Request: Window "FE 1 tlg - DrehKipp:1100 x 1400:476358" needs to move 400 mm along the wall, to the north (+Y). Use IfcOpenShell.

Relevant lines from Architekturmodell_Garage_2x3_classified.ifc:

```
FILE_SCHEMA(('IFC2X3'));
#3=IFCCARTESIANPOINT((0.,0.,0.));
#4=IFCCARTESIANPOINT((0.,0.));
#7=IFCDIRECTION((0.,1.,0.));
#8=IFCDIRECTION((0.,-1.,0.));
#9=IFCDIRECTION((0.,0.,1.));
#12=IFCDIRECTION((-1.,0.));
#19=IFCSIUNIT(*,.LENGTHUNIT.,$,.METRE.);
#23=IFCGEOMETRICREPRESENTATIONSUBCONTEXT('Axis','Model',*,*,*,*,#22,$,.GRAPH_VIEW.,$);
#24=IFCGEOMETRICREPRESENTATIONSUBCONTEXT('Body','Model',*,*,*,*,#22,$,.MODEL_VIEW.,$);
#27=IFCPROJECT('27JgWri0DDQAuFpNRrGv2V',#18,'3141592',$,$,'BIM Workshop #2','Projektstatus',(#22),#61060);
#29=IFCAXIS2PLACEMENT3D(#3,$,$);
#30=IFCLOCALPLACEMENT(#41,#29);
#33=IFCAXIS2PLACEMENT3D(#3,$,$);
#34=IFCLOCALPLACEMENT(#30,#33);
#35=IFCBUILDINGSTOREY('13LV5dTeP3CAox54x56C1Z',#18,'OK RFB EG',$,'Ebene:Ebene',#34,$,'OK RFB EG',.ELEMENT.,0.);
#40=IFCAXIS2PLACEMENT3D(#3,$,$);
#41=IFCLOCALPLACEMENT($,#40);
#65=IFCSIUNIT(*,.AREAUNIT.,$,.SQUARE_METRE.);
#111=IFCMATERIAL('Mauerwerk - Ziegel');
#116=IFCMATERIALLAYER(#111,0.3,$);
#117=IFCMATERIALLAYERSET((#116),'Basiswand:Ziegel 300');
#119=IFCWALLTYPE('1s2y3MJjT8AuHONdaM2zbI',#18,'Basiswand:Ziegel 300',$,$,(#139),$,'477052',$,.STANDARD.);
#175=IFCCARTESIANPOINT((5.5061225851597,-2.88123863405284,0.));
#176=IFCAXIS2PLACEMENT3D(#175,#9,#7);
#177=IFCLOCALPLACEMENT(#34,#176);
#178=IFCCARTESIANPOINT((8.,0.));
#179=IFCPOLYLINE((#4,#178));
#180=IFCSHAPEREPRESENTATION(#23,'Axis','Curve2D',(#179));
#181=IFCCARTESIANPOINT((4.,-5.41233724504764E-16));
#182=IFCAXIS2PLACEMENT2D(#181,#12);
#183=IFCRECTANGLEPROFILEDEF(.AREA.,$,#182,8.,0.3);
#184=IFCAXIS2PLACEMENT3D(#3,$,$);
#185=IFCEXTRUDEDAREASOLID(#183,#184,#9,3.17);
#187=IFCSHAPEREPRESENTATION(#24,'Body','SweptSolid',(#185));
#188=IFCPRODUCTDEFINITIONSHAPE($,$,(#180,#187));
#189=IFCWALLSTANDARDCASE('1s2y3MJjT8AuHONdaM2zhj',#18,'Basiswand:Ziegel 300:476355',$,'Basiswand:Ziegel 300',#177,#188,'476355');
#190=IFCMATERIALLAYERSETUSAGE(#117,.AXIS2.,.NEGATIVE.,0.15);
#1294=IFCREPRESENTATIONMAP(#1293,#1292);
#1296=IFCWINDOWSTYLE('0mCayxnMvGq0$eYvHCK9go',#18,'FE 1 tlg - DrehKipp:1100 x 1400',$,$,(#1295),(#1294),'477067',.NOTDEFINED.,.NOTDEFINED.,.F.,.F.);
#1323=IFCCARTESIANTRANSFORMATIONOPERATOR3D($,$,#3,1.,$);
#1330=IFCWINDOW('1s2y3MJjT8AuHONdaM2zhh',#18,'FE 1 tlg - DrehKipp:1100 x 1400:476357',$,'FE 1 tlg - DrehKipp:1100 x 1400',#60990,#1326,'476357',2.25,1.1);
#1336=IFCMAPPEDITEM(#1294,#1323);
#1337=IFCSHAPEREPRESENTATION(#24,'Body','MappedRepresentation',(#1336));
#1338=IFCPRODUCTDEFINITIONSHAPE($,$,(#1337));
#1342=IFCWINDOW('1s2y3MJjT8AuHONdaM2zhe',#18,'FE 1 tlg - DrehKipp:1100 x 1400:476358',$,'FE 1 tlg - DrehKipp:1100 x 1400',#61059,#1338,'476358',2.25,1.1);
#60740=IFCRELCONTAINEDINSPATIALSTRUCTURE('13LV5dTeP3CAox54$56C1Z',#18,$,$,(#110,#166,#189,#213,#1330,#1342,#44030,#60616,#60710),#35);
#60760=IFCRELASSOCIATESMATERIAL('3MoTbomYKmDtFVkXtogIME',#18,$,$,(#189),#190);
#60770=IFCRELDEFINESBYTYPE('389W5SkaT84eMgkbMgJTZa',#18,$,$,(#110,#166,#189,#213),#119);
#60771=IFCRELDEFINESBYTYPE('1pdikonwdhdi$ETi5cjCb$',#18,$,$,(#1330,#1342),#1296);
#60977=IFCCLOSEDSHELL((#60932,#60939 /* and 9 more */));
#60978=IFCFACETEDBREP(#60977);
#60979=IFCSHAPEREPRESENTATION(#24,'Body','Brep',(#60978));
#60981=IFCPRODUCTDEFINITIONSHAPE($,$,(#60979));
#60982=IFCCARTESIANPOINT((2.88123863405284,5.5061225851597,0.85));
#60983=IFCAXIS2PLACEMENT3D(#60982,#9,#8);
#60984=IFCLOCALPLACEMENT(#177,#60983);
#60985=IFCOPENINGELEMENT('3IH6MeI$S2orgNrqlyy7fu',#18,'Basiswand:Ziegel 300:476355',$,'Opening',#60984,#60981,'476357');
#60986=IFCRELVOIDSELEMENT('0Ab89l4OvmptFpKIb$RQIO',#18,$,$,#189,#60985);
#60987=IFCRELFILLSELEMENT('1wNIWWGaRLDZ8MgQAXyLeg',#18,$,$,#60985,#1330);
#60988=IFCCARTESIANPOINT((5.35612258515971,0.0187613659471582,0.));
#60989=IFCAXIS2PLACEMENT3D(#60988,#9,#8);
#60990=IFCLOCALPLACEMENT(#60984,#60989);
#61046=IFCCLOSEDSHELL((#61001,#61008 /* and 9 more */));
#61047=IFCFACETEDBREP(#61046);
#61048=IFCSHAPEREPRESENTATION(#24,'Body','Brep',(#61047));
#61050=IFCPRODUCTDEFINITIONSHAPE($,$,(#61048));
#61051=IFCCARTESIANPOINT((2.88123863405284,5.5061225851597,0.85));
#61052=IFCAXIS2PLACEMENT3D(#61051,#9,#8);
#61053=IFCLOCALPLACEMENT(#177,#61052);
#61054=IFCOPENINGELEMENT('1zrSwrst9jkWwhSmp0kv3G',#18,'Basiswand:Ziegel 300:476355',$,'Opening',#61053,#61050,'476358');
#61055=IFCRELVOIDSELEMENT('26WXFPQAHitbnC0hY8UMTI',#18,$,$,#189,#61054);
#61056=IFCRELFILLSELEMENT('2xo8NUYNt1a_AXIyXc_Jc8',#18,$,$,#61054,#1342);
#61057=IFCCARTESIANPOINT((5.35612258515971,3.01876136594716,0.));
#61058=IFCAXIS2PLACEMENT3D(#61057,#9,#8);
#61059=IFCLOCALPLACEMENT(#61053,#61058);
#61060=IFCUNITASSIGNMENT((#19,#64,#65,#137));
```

```python
import ifcopenshell
import ifcopenshell.api.geometry
import ifcopenshell.util.placement
import ifcopenshell.util.unit

model = ifcopenshell.open("Architekturmodell_Garage_2x3_classified.ifc")
unit_scale = ifcopenshell.util.unit.calculate_unit_scale(model)

window = model.by_guid("1s2y3MJjT8AuHONdaM2zhe")
opening = window.FillsVoids[0].RelatingOpeningElement
wall = opening.VoidsElements[0].RelatingBuildingElement

wall_matrix = ifcopenshell.util.placement.get_local_placement(wall.ObjectPlacement)
shift = wall_matrix[:3, 0] * 0.4 / unit_scale
before = ifcopenshell.util.placement.get_local_placement(window.ObjectPlacement)[:3, 3].copy()

# The window is placed relative to its opening, so it follows when the opening moves.
matrix = ifcopenshell.util.placement.get_local_placement(opening.ObjectPlacement)
matrix[:3, 3] += shift
ifcopenshell.api.geometry.edit_object_placement(
    model, product=opening, matrix=matrix, is_si=False, should_transform_children=True
)

after = ifcopenshell.util.placement.get_local_placement(window.ObjectPlacement)[:3, 3]
print("window moved by", (after - before).round(3) + 0.0)

model.write("Architekturmodell_Garage_2x3_classified_rev.ifc")
```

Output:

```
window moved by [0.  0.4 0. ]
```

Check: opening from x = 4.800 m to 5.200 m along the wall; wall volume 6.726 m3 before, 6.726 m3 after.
